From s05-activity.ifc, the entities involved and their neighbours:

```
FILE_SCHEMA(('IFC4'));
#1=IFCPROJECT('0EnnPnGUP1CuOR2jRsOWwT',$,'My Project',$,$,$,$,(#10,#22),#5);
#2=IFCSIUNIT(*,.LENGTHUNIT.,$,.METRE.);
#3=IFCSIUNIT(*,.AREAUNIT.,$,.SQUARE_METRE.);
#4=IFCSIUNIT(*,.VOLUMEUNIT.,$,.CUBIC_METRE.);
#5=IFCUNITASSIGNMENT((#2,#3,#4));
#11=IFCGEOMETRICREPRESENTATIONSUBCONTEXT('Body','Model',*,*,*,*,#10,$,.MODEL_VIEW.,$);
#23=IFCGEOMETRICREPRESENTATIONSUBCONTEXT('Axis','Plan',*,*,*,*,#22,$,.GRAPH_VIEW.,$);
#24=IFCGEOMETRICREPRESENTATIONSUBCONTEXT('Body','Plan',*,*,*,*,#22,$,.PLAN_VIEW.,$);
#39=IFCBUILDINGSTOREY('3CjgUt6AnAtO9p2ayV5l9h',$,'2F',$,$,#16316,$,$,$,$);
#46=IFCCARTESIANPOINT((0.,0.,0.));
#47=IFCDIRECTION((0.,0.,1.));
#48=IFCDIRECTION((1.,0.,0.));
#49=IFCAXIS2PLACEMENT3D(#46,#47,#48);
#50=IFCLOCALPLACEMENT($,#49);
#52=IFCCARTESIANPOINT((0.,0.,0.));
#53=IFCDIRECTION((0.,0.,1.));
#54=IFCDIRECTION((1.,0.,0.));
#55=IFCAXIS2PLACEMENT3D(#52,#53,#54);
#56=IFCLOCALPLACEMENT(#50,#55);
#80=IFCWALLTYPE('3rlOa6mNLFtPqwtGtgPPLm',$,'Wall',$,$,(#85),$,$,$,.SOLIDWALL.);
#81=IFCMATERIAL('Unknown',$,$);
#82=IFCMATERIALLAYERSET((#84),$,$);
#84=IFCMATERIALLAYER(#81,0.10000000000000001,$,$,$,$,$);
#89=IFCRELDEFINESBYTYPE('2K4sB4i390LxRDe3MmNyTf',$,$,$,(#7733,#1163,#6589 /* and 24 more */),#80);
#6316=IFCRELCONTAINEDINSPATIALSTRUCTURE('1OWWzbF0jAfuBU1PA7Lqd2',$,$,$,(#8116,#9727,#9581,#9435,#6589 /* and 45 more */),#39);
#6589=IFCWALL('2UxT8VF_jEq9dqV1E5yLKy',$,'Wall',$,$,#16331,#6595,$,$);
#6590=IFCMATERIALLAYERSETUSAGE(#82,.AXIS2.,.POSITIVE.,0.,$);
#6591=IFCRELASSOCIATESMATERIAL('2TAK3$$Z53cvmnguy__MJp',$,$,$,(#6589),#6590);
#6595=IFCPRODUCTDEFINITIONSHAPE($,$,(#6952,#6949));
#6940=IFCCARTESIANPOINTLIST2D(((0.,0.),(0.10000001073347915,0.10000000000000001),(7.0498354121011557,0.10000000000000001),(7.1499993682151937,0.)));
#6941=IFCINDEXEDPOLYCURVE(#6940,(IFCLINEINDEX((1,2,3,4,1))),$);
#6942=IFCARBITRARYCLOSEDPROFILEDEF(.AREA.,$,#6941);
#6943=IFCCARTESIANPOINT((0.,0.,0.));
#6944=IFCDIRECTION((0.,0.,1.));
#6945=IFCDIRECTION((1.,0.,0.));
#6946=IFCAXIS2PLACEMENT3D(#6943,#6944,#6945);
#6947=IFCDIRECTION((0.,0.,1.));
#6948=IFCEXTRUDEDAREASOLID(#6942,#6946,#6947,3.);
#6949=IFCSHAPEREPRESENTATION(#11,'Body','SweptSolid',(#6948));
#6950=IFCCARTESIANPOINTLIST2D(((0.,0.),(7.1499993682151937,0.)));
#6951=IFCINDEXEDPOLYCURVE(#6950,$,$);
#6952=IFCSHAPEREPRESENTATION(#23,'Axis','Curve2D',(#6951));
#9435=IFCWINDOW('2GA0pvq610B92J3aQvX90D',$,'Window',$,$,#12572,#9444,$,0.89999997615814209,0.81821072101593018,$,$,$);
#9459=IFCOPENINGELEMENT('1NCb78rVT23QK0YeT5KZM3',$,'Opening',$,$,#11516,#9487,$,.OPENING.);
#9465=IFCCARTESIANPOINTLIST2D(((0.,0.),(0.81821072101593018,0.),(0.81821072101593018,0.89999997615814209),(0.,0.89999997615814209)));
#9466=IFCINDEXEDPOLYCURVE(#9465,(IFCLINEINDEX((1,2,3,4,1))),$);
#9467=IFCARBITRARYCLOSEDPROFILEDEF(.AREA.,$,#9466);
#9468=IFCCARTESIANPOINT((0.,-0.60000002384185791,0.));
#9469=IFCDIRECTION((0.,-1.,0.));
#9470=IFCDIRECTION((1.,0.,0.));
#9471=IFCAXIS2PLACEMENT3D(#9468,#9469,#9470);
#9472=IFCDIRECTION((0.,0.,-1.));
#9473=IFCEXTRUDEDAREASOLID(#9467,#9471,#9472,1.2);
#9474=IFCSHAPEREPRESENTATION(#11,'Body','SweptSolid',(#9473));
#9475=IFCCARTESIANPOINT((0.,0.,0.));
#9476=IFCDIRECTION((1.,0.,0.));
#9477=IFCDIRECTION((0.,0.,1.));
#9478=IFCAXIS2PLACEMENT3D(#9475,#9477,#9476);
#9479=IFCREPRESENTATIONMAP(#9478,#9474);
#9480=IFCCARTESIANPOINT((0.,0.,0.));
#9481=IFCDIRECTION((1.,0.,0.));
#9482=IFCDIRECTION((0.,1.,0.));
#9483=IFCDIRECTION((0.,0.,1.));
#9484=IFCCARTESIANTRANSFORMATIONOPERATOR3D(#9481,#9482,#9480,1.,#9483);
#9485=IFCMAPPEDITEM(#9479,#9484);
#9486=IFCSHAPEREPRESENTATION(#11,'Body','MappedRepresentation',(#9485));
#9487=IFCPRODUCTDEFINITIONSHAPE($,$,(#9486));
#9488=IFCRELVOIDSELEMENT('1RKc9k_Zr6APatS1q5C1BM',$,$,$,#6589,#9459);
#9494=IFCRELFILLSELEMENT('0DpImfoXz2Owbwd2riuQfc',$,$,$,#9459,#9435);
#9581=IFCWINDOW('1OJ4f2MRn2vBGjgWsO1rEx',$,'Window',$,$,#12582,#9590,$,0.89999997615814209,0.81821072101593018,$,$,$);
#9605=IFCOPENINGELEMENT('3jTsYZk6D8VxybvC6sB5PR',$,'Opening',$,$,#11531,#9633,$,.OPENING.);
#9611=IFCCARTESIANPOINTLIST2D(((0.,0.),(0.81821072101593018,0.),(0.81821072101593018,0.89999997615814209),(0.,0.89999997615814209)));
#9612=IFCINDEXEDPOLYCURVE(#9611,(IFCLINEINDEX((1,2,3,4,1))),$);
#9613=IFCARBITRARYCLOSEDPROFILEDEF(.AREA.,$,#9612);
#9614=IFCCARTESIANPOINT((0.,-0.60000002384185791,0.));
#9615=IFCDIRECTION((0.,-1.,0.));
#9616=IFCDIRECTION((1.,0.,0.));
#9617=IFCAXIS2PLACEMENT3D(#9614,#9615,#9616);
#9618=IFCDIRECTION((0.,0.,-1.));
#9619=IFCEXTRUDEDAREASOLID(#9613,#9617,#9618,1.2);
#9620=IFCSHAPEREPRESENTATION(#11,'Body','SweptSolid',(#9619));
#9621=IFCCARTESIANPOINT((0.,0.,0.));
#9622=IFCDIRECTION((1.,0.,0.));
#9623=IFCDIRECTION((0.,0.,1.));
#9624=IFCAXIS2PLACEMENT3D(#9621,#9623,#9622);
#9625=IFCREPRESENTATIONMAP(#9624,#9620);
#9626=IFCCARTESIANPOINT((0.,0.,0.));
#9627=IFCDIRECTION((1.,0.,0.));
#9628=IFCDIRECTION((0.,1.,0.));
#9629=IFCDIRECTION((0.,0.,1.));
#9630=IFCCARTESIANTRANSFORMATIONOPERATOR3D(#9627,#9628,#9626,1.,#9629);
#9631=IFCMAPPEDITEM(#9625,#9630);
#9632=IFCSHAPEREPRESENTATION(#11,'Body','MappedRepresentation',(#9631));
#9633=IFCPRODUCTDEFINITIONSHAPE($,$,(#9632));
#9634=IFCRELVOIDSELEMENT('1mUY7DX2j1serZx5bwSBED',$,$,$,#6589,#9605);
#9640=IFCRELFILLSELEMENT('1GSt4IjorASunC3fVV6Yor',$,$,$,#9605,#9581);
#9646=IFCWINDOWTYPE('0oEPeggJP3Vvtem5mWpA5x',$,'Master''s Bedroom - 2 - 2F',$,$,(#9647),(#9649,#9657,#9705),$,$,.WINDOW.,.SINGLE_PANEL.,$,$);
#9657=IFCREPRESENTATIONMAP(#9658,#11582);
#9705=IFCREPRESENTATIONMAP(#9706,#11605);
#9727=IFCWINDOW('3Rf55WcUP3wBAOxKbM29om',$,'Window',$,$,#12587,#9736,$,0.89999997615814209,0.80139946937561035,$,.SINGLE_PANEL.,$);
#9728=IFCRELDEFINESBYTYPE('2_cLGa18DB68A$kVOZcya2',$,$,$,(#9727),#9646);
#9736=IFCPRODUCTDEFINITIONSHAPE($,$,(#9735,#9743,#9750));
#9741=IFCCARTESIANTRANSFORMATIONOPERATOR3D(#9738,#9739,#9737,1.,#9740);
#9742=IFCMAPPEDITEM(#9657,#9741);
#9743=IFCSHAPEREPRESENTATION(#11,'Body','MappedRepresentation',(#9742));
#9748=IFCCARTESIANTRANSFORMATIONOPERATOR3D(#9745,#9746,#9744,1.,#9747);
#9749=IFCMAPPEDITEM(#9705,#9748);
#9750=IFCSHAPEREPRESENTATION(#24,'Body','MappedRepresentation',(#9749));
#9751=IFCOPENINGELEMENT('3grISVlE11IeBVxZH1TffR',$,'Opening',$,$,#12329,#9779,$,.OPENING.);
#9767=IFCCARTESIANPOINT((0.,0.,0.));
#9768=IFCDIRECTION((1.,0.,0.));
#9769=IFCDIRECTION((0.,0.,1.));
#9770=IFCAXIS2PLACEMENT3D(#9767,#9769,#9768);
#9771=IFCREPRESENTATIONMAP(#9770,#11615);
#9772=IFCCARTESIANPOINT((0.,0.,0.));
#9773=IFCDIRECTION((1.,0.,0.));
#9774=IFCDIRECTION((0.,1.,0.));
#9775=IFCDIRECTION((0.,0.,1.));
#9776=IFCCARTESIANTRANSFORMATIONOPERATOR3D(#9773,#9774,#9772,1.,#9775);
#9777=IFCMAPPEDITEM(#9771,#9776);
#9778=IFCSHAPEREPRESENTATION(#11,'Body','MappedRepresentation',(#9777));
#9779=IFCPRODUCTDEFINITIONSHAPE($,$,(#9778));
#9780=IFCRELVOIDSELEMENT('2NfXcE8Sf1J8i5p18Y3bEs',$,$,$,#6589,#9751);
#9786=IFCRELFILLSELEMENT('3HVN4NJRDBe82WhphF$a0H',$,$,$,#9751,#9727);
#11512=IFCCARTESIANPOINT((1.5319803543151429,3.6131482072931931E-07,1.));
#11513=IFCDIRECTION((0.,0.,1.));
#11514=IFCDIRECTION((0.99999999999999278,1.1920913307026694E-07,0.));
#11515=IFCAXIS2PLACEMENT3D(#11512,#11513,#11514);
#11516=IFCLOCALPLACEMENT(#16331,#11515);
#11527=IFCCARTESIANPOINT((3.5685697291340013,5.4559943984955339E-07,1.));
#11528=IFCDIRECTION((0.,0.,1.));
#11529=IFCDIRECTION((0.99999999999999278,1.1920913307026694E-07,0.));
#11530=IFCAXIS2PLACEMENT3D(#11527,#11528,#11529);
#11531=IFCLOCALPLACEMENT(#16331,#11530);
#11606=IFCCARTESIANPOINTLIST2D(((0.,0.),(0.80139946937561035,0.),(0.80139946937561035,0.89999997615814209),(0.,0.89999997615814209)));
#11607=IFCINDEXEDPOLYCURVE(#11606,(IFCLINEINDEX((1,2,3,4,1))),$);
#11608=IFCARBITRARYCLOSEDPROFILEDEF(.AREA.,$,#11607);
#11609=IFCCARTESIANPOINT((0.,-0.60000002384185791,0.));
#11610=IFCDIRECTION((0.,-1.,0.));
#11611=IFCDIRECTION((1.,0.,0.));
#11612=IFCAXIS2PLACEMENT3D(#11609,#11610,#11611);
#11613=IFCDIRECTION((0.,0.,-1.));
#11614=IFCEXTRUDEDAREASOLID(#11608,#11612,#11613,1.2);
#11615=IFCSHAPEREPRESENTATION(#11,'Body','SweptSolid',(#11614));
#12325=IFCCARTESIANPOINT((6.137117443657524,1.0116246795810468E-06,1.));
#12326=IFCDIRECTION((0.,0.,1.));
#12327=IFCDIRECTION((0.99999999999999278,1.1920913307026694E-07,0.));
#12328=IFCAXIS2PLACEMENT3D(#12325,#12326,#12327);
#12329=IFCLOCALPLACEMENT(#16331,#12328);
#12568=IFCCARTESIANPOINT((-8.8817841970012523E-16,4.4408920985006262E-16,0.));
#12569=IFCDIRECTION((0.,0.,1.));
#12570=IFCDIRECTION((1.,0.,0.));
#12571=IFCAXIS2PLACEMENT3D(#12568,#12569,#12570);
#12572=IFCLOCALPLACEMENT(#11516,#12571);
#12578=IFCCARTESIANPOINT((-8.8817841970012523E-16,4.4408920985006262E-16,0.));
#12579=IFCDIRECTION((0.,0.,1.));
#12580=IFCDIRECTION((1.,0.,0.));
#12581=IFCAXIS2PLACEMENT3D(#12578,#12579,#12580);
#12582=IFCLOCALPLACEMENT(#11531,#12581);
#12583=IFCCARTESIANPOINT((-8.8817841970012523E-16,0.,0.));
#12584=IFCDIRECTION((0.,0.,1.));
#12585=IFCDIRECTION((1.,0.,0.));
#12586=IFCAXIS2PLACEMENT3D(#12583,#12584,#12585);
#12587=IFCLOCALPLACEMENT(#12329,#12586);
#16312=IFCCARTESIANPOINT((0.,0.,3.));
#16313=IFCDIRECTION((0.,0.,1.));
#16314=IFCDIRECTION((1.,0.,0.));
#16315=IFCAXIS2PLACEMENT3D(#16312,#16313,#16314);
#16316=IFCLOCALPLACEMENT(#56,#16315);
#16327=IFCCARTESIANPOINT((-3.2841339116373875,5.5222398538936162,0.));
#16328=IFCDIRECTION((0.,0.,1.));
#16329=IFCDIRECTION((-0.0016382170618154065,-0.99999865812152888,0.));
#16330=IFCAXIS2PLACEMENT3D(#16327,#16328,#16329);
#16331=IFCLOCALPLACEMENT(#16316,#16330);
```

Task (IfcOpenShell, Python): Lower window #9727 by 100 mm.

```python
import numpy as np
import ifcopenshell
import ifcopenshell.api.geometry
import ifcopenshell.util.placement
import ifcopenshell.util.unit

model = ifcopenshell.open("s05-activity.ifc")
unit_scale = ifcopenshell.util.unit.calculate_unit_scale(model)

window = model.by_guid("3Rf55WcUP3wBAOxKbM29om")
opening = window.FillsVoids[0].RelatingOpeningElement
dz = -0.1 / unit_scale

shift = np.array([0.0, 0.0, dz])
# The window is placed relative to its opening, so it follows when the opening moves.
matrix = ifcopenshell.util.placement.get_local_placement(opening.ObjectPlacement)
matrix[:3, 3] += shift
ifcopenshell.api.geometry.edit_object_placement(
    model, product=opening, matrix=matrix, is_si=False, should_transform_children=True
)

print(f"moved by {dz * unit_scale:+.3f} m")

model.write("s05-activity_edited.ifc")
```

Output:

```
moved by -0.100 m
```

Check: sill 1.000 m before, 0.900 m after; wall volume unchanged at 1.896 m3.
